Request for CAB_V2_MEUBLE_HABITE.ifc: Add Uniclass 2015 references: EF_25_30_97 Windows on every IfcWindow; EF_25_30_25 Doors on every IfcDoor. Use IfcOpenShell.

First a look at what the model holds.

```python
import ifcopenshell

model = ifcopenshell.open("CAB_V2_MEUBLE_HABITE.ifc")
print(model.schema)
print("classifications:", [c.Name for c in model.by_type("IfcClassification")])
for ifc_class in ("IfcDoor", "IfcRoof", "IfcStair", "IfcWall", "IfcWindow"):
    print(ifc_class, len(model.by_type(ifc_class)))
```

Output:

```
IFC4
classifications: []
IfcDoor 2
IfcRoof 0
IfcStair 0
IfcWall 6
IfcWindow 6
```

```python
import ifcopenshell
import ifcopenshell.api.classification

model = ifcopenshell.open("CAB_V2_MEUBLE_HABITE.ifc")

system = ifcopenshell.api.classification.add_classification(model, classification="Uniclass 2015")

codes = {
    "IfcWindow": ("EF_25_30_97", "Windows"),
    "IfcDoor": ("EF_25_30_25", "Doors"),
}
for ifc_class, (code, name) in codes.items():
    products = model.by_type(ifc_class)
    ifcopenshell.api.classification.add_reference(
        model, products=products, classification=system, identification=code, name=name
    )
    print(code, len(products))

model.write("CAB_V2_MEUBLE_HABITE_rev.ifc")
```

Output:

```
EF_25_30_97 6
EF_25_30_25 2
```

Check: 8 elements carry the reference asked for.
